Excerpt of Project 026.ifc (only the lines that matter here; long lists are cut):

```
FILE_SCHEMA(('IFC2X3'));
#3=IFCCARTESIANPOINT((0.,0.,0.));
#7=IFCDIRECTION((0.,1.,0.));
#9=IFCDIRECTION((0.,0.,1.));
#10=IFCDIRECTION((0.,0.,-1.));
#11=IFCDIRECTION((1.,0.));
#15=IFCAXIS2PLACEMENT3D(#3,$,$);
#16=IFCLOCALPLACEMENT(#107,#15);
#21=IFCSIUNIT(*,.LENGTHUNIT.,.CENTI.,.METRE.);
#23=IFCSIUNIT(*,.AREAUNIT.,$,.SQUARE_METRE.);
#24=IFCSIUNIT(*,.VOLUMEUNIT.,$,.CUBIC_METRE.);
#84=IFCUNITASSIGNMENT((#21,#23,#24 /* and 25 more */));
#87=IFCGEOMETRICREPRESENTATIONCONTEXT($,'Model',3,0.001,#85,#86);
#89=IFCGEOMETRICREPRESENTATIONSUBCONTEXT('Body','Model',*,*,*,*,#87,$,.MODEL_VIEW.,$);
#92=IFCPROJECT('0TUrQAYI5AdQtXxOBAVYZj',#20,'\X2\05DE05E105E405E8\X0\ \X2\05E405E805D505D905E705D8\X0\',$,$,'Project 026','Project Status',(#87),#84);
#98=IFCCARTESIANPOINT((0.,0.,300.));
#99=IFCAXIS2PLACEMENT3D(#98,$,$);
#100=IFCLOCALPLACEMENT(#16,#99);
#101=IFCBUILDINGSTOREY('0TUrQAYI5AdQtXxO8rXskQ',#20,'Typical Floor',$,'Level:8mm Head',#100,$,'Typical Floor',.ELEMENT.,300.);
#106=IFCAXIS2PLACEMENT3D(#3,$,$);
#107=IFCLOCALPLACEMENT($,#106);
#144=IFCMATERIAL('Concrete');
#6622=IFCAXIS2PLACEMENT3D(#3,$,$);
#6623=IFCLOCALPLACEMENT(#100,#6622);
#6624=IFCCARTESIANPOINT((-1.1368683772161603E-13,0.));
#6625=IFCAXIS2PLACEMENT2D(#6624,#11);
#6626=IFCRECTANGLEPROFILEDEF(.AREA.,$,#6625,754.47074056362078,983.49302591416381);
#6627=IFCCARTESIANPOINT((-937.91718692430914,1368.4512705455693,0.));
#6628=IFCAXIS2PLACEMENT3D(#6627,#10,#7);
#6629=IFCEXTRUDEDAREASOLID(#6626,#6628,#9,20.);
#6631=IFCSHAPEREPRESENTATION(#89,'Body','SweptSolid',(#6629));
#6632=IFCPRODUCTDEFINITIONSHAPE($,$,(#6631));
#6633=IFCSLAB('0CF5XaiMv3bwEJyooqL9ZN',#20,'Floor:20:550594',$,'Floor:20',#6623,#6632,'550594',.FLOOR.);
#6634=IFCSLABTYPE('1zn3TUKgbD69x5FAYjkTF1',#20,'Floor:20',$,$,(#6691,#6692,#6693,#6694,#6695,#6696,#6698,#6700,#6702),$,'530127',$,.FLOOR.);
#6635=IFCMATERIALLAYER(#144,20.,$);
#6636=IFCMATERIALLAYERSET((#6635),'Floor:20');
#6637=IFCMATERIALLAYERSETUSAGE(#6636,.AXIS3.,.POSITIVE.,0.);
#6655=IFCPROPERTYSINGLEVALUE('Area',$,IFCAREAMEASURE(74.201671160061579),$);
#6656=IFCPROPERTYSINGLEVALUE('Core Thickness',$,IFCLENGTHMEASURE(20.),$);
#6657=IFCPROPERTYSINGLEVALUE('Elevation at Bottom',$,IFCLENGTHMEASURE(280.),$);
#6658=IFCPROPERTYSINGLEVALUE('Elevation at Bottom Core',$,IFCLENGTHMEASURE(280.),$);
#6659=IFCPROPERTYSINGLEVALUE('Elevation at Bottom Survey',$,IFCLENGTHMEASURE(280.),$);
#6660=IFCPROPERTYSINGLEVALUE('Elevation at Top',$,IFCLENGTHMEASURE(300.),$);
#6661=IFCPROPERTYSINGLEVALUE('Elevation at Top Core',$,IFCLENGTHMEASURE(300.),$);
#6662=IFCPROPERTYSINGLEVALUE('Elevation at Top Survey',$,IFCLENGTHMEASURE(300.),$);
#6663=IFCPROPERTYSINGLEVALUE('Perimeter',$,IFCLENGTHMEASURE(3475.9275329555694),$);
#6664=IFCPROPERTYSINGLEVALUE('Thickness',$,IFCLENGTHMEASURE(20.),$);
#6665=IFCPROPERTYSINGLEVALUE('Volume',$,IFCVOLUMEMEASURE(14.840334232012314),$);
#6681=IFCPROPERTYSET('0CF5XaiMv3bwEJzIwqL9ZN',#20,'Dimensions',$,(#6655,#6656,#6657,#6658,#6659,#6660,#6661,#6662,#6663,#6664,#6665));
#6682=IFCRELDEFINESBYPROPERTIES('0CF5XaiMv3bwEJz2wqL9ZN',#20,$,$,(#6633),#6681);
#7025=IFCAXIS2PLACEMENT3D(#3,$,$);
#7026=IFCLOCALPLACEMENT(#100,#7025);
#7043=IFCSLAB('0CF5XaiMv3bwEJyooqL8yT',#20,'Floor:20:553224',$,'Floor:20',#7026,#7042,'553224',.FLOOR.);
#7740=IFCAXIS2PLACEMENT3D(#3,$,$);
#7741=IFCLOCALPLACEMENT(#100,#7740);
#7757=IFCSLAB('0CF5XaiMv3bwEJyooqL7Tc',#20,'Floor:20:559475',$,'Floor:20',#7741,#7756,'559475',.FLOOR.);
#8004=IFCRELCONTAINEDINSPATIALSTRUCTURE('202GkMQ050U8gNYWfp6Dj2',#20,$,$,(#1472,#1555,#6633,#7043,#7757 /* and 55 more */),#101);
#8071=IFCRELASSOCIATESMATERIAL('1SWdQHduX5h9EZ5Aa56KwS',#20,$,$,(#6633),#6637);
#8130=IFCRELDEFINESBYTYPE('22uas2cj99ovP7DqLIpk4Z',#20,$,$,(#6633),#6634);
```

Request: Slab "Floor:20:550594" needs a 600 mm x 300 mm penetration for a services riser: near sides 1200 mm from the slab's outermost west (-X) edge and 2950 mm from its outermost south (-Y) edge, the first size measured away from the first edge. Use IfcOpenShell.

```python
import numpy as np
import ifcopenshell
import ifcopenshell.api.feature
import ifcopenshell.api.geometry
import ifcopenshell.api.pset
import ifcopenshell.api.root
import ifcopenshell.geom
import ifcopenshell.util.element
import ifcopenshell.util.placement
import ifcopenshell.util.representation
import ifcopenshell.util.shape
import ifcopenshell.util.unit

model = ifcopenshell.open("Project 026.ifc")
unit_scale = ifcopenshell.util.unit.calculate_unit_scale(model)
area_scale = ifcopenshell.util.unit.calculate_unit_scale(model, "AREAUNIT")
volume_scale = ifcopenshell.util.unit.calculate_unit_scale(model, "VOLUMEUNIT")
settings = ifcopenshell.geom.settings()


def volume(element):
    """Net volume in cubic metres, openings subtracted."""
    shape = ifcopenshell.geom.create_shape(settings, element)
    return ifcopenshell.util.shape.get_volume(shape.geometry)


slab = model.by_guid("0CF5XaiMv3bwEJyooqL9ZN")
before = volume(slab)

# Extent in the slab's own axes, in metres. The edges named are its -X and -Y sides.
slab_shape = ifcopenshell.geom.create_shape(settings, slab)
vertices = ifcopenshell.util.shape.get_vertices(slab_shape.geometry)
x_min, y_min, bottom = vertices.min(axis=0)
top = vertices[:, 2].max()

opening = ifcopenshell.api.root.create_entity(model, ifc_class="IfcOpeningElement", name="Services riser opening")
context = ifcopenshell.util.representation.get_context(model, "Model", "Body", "MODEL_VIEW")
width, depth = 0.6, 0.3
outline = [(0.0, 0.0), (width, 0.0), (width, depth), (0.0, depth), (0.0, 0.0)]
# Overshoot both faces by 50 mm so the cut is clean.
shape = ifcopenshell.api.geometry.add_slab_representation(
    model, context=context, depth=top - bottom + 0.1, polyline=outline
)
ifcopenshell.api.geometry.assign_representation(model, product=opening, representation=shape)

matrix = ifcopenshell.util.placement.get_local_placement(slab.ObjectPlacement)
matrix[:, 3] = matrix @ np.append(np.array([x_min + 1.2, y_min + 2.95, bottom - 0.05]) / unit_scale, 1.0)
ifcopenshell.api.geometry.edit_object_placement(model, product=opening, matrix=matrix, is_si=False)
ifcopenshell.api.feature.add_feature(model, feature=opening, element=slab)

after = volume(slab)

# Update the slab's stored quantities.
pset = model.by_id(ifcopenshell.util.element.get_pset(slab, "Dimensions", should_inherit=False)["id"])
ifcopenshell.api.pset.edit_pset(model, pset=pset, properties={
    "Area": model.create_entity("IfcAreaMeasure", after / (top - bottom) / area_scale),
    "Volume": model.create_entity("IfcVolumeMeasure", after / volume_scale),
})

print(f"slab volume {before:.3f} -> {after:.3f} m3")

model.write("Project 026-out.ifc")
```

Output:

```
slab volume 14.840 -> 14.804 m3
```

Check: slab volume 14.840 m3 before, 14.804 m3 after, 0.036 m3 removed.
